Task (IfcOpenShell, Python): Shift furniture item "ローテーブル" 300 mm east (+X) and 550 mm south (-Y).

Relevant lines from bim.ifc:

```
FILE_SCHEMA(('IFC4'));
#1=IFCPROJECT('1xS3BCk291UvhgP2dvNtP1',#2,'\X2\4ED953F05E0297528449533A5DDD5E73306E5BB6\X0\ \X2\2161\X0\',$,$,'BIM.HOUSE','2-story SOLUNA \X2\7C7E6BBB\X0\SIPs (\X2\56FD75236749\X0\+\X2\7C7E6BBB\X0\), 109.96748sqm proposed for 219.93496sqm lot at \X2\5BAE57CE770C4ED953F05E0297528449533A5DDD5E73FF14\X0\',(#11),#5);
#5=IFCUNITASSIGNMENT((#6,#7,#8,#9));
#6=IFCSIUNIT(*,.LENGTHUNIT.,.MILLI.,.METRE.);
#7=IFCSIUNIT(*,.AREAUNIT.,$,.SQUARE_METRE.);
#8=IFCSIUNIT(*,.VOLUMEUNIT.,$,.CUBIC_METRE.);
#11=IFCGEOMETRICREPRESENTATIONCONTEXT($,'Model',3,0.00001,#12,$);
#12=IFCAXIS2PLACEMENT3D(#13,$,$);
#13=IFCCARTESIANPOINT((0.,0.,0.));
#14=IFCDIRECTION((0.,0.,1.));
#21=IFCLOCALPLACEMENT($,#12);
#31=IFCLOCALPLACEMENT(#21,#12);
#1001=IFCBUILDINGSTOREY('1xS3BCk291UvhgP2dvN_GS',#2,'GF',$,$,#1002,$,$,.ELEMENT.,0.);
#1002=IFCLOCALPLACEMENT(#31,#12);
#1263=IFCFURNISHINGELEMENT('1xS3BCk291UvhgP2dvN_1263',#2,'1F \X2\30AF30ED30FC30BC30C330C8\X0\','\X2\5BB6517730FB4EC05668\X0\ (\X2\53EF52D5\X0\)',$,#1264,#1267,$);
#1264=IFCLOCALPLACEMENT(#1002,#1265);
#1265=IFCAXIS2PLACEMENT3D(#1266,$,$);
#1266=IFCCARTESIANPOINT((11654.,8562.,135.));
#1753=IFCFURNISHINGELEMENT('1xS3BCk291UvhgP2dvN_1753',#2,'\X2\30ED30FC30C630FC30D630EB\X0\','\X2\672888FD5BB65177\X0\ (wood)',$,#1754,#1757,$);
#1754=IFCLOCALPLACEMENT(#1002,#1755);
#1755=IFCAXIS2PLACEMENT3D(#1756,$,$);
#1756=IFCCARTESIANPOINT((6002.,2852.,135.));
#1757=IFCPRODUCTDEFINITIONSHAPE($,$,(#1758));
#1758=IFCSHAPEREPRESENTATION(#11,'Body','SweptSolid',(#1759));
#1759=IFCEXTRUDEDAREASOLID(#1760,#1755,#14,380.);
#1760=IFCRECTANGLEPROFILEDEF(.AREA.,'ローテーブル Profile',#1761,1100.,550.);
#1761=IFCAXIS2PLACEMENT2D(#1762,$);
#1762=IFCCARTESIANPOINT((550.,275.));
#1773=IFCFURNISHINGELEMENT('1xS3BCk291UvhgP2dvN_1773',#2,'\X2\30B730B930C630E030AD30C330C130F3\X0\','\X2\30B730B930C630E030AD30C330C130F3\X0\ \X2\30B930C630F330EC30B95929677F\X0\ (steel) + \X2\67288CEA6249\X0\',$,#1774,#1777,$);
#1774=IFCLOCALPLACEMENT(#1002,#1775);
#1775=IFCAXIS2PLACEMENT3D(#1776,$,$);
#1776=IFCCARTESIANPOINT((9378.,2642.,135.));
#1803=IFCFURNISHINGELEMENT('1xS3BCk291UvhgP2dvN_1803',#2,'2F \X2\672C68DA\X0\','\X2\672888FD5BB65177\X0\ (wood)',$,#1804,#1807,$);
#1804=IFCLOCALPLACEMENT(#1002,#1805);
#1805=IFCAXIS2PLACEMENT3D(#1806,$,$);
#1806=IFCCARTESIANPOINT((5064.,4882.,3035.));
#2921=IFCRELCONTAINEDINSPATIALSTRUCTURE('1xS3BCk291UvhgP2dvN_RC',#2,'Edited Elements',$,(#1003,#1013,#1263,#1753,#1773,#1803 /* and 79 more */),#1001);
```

```python
import ifcopenshell
import ifcopenshell.api.geometry
import ifcopenshell.util.placement
import ifcopenshell.util.unit

model = ifcopenshell.open("bim.ifc")
unit_scale = ifcopenshell.util.unit.calculate_unit_scale(model)

item = model.by_guid("1xS3BCk291UvhgP2dvN_1753")
matrix = ifcopenshell.util.placement.get_local_placement(item.ObjectPlacement)
matrix[0, 3] += 0.3 / unit_scale
matrix[1, 3] -= 0.55 / unit_scale
ifcopenshell.api.geometry.edit_object_placement(model, product=item, matrix=matrix, is_si=False)

print(ifcopenshell.util.placement.get_local_placement(item.ObjectPlacement).round(3) + 0.0)

model.write("bim_updated.ifc")
```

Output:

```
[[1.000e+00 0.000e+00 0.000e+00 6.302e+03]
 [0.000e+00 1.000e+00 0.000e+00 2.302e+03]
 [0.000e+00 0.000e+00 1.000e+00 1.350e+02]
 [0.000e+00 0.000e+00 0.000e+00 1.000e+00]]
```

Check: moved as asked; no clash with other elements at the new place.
